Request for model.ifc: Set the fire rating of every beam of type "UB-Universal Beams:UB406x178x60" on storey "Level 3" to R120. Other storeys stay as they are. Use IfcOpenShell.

First a look at what the model holds.

```python
import ifcopenshell
import ifcopenshell.util.element

model = ifcopenshell.open("model.ifc")
print(model.schema)
storey = next(s for s in model.by_type("IfcBuildingStorey") if s.Name == "Level 3")
beams = [e for e in ifcopenshell.util.element.get_decomposition(storey) if e.is_a("IfcBeam")]
seen = {}
for e in beams:
    element_type = ifcopenshell.util.element.get_type(e)
    key = (element_type.Name if element_type != e and element_type else None, ifcopenshell.util.element.get_pset(e, "Pset_BeamCommon", "FireRating"))
    seen[key] = seen.get(key, 0) + 1
for (name, value), count in sorted(seen.items(), key=str):
    print(count, "x", name, "|", value)
```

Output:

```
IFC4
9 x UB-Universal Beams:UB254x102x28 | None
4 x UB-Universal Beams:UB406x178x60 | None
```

```python
import ifcopenshell
import ifcopenshell.api.pset
import ifcopenshell.util.element

model = ifcopenshell.open("model.ifc")

storey = next(s for s in model.by_type("IfcBuildingStorey") if s.Name == "Level 3")
beams = [e for e in ifcopenshell.util.element.get_decomposition(storey) if e.is_a("IfcBeam")]

count = 0
for e in beams:
    element_type = ifcopenshell.util.element.get_type(e)
    if element_type in (None, e) or element_type.Name != "UB-Universal Beams:UB406x178x60":
        continue
    # add_pset returns the element's existing set when there is one.
    pset = ifcopenshell.api.pset.add_pset(model, product=e, name="Pset_BeamCommon")
    ifcopenshell.api.pset.edit_pset(model, pset=pset, properties={"FireRating": "R120"})
    count += 1

print(count, "beams updated")

model.write("model_updated.ifc")
```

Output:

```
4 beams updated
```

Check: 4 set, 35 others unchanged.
